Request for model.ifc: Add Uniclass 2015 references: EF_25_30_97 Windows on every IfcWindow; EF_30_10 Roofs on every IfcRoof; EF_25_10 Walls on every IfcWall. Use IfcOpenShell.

First a look at what the model holds.

```python
import ifcopenshell

model = ifcopenshell.open("model.ifc")
print(model.schema)
print("classifications:", [c.Name for c in model.by_type("IfcClassification")])
for ifc_class in ("IfcDoor", "IfcRoof", "IfcStair", "IfcWall", "IfcWindow"):
    print(ifc_class, len(model.by_type(ifc_class)))
```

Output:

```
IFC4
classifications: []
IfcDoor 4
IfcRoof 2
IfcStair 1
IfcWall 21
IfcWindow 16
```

```python
import ifcopenshell
import ifcopenshell.api.classification

model = ifcopenshell.open("model.ifc")

system = ifcopenshell.api.classification.add_classification(model, classification="Uniclass 2015")

codes = {
    "IfcWindow": ("EF_25_30_97", "Windows"),
    "IfcRoof": ("EF_30_10", "Roofs"),
    "IfcWall": ("EF_25_10", "Walls"),
}
for ifc_class, (code, name) in codes.items():
    products = model.by_type(ifc_class)
    ifcopenshell.api.classification.add_reference(
        model, products=products, classification=system, identification=code, name=name
    )
    print(code, len(products))

model.write("model_v2.ifc")
```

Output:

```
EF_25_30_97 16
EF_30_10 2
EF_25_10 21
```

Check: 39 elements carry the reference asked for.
